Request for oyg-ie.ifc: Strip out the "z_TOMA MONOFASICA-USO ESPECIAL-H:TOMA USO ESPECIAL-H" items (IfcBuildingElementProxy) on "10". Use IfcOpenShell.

First a look at what the model holds.

```python
import ifcopenshell
import ifcopenshell.util.element

model = ifcopenshell.open("oyg-ie.ifc")
print(model.schema)
storey = next(s for s in model.by_type("IfcBuildingStorey") if s.Name == "10")
proxies = [e for e in ifcopenshell.util.element.get_decomposition(storey) if e.is_a("IfcBuildingElementProxy")]
seen = {}
for e in proxies:
    element_type = ifcopenshell.util.element.get_type(e)
    name = element_type.Name if element_type not in (None, e) else None
    seen[name] = seen.get(name, 0) + 1
for name, count in sorted(seen.items(), key=str):
    print(count, "x", name)
```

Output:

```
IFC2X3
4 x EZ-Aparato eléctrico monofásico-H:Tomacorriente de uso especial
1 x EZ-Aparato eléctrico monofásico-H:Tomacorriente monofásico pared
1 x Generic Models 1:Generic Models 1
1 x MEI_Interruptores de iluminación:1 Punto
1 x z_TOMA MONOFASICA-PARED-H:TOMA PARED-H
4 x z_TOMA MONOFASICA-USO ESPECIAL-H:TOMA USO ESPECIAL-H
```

```python
import ifcopenshell
import ifcopenshell.api.root
import ifcopenshell.util.element

model = ifcopenshell.open("oyg-ie.ifc")

storey = next(s for s in model.by_type("IfcBuildingStorey") if s.Name == "10")
proxies = [e for e in ifcopenshell.util.element.get_decomposition(storey) if e.is_a("IfcBuildingElementProxy")]
targets = [e for e in proxies if (t := ifcopenshell.util.element.get_type(e)) not in (None, e) and t.Name == "z_TOMA MONOFASICA-USO ESPECIAL-H:TOMA USO ESPECIAL-H"]

for e in targets:
    ifcopenshell.api.root.remove_product(model, product=e)
print(len(targets), "removed")

model.write("oyg-ie_edited.ifc")
```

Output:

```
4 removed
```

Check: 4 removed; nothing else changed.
